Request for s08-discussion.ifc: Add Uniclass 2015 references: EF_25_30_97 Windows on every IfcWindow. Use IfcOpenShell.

First a look at what the model holds.

```python
import ifcopenshell

model = ifcopenshell.open("s08-discussion.ifc")
print(model.schema)
print("classifications:", [c.Name for c in model.by_type("IfcClassification")])
for ifc_class in ("IfcDoor", "IfcRoof", "IfcStair", "IfcWall", "IfcWindow"):
    print(ifc_class, len(model.by_type(ifc_class)))
```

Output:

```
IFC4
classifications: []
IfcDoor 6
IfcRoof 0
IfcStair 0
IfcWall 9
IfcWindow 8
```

```python
import ifcopenshell
import ifcopenshell.api.classification

model = ifcopenshell.open("s08-discussion.ifc")

system = ifcopenshell.api.classification.add_classification(model, classification="Uniclass 2015")

codes = {
    "IfcWindow": ("EF_25_30_97", "Windows"),
}
for ifc_class, (code, name) in codes.items():
    products = model.by_type(ifc_class)
    ifcopenshell.api.classification.add_reference(
        model, products=products, classification=system, identification=code, name=name
    )
    print(code, len(products))

model.write("s08-discussion_rev.ifc")
```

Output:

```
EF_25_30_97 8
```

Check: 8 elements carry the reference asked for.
